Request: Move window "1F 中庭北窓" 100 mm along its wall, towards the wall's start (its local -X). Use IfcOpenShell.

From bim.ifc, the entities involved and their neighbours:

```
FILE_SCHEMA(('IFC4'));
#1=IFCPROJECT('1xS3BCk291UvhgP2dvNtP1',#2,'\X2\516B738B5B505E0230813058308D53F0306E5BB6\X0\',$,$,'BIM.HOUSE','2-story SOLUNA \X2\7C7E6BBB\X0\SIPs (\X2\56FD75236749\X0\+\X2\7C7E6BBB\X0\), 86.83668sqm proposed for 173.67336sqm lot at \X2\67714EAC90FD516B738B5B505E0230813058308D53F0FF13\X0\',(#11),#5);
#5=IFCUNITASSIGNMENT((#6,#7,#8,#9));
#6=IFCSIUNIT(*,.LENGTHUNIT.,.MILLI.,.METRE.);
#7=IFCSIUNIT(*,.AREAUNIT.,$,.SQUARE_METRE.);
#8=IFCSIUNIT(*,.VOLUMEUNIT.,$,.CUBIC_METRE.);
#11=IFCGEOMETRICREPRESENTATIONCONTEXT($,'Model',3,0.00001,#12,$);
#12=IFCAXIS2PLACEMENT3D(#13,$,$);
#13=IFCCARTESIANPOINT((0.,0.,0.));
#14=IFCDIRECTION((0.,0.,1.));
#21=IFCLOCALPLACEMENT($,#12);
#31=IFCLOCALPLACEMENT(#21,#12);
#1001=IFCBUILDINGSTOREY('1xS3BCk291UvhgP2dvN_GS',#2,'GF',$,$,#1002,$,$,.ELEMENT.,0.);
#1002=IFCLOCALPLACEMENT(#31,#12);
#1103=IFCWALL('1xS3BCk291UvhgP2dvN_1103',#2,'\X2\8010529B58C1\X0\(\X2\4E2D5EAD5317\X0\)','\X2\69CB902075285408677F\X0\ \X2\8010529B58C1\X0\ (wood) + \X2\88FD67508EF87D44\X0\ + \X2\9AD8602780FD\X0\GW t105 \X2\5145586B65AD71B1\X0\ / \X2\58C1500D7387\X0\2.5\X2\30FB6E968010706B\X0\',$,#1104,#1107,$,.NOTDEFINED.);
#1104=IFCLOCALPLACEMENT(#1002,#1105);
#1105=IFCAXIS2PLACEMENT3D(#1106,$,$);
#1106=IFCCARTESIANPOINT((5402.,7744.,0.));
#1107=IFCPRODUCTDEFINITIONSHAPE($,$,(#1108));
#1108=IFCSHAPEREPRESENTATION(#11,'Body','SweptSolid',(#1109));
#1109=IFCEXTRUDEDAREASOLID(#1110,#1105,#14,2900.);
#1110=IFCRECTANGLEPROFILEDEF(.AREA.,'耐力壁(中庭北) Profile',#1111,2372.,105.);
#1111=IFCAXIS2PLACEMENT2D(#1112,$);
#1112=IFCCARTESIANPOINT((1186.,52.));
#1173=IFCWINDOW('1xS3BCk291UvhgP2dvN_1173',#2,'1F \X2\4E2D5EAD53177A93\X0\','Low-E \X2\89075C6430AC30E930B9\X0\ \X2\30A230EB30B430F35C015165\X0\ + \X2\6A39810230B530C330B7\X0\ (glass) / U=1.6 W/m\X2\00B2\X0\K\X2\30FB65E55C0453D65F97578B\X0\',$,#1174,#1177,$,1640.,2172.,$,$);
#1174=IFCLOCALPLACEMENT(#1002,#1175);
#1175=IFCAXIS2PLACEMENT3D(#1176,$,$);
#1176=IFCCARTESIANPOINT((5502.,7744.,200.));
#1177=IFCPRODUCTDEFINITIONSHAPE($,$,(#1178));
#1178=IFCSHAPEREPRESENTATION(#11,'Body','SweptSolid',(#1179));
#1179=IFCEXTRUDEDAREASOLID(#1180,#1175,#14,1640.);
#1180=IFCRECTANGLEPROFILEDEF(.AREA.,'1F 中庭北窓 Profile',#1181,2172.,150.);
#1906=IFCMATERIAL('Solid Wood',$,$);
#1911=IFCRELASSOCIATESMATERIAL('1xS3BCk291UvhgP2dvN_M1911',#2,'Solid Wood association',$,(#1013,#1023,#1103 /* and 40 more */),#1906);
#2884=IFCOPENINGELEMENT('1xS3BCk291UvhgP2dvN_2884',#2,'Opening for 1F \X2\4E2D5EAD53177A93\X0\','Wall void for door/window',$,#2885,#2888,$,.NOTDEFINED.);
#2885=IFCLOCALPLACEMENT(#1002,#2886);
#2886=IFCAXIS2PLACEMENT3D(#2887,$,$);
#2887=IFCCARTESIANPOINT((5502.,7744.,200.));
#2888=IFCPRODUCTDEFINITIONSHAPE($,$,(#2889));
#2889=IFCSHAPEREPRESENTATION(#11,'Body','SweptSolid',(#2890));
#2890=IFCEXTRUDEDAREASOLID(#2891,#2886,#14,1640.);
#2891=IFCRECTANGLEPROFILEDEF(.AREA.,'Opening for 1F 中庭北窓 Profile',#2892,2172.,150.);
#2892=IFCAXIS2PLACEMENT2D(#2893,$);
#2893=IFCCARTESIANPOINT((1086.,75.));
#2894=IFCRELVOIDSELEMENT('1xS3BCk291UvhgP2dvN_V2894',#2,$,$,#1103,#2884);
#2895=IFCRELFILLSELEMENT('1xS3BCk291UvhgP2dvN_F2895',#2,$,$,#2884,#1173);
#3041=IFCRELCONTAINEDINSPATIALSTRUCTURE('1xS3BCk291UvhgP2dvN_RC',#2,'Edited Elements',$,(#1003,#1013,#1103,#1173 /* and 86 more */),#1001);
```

```python
import ifcopenshell
import ifcopenshell.api.geometry
import ifcopenshell.util.placement
import ifcopenshell.util.unit

model = ifcopenshell.open("bim.ifc")
unit_scale = ifcopenshell.util.unit.calculate_unit_scale(model)

window = model.by_id(1173)
opening = window.FillsVoids[0].RelatingOpeningElement
wall = opening.VoidsElements[0].RelatingBuildingElement

wall_matrix = ifcopenshell.util.placement.get_local_placement(wall.ObjectPlacement)
shift = wall_matrix[:3, 0] * -0.1 / unit_scale
before = ifcopenshell.util.placement.get_local_placement(window.ObjectPlacement)[:3, 3].copy()

# The window is not placed relative to its opening, so move both.
for product in (opening, window):
    matrix = ifcopenshell.util.placement.get_local_placement(product.ObjectPlacement)
    matrix[:3, 3] += shift
    ifcopenshell.api.geometry.edit_object_placement(model, product=product, matrix=matrix, is_si=False)

after = ifcopenshell.util.placement.get_local_placement(window.ObjectPlacement)[:3, 3]
print("window moved by", (after - before).round(3) + 0.0)

model.write("bim-out.ifc")
```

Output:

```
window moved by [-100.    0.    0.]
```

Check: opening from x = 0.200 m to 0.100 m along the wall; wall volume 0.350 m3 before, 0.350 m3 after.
